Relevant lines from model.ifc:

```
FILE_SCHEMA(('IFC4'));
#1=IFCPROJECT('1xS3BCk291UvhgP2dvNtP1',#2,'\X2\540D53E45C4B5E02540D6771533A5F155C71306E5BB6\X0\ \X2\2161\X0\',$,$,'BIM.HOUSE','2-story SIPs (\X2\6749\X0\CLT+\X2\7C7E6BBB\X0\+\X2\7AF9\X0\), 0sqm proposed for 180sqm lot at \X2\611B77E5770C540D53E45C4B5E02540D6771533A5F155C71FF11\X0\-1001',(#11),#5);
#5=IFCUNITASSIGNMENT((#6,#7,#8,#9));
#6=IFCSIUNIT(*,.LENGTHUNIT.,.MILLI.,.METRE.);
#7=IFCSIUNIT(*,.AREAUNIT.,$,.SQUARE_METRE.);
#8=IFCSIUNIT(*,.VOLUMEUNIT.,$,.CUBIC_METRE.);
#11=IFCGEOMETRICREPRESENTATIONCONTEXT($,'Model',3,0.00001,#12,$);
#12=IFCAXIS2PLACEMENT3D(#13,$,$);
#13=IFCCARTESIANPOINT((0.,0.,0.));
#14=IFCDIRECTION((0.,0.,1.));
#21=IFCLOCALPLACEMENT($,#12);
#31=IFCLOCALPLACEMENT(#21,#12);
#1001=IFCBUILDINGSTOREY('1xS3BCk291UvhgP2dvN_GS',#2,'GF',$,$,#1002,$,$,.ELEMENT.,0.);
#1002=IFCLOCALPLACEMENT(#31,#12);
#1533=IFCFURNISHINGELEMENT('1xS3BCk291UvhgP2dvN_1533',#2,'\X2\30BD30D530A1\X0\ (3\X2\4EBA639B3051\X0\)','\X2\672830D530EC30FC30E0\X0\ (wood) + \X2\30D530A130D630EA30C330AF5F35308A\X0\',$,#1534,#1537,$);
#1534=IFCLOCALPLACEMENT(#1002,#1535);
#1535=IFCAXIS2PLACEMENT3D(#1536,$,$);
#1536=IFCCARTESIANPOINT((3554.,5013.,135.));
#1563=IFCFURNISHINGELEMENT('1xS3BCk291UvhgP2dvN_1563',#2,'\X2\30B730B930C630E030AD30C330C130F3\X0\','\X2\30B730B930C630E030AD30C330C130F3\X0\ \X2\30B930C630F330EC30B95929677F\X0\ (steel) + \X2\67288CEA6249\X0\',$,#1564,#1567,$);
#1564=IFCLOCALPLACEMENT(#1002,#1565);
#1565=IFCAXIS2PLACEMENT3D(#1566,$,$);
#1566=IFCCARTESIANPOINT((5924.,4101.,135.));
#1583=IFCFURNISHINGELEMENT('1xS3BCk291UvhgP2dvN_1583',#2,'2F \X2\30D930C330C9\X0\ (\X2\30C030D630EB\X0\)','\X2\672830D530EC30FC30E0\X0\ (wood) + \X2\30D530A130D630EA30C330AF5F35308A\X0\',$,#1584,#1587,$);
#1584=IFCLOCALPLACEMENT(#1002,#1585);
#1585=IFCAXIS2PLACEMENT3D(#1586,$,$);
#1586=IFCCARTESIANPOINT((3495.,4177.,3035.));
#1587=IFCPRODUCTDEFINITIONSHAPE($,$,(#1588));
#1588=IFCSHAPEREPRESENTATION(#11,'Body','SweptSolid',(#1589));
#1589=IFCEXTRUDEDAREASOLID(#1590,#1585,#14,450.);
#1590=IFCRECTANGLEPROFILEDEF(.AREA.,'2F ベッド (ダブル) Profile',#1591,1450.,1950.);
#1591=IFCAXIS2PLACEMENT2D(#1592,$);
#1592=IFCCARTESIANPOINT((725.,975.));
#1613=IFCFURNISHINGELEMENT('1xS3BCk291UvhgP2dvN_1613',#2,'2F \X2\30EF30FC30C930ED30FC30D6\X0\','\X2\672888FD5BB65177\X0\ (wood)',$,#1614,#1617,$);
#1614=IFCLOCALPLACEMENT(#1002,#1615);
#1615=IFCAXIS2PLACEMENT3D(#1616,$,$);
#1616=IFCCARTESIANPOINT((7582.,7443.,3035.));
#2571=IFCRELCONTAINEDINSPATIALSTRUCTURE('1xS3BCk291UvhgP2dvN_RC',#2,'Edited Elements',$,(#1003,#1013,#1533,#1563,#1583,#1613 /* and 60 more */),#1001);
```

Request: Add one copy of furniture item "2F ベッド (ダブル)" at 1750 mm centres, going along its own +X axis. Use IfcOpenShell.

```python
import ifcopenshell
import ifcopenshell.api.geometry
import ifcopenshell.api.root
import ifcopenshell.util.element
import ifcopenshell.util.placement
import ifcopenshell.util.unit

model = ifcopenshell.open("model.ifc")
unit_scale = ifcopenshell.util.unit.calculate_unit_scale(model)


def reuse_history(source, copy):
    """copy_class also copies each property set's owner history, people and application; keep the originals."""
    for rel in copy.IsDefinedBy:
        if rel.is_a("IfcRelDefinesByProperties") and (history := rel.RelatingPropertyDefinition.OwnerHistory):
            rel.RelatingPropertyDefinition.OwnerHistory = source.OwnerHistory
            ifcopenshell.util.element.remove_deep2(model, history)


source = model.by_guid("1xS3BCk291UvhgP2dvN_1583")
base = ifcopenshell.util.placement.get_local_placement(source.ObjectPlacement)
step = base[:3, 0] * 1.75 / unit_scale

for i in range(1, 2):
    copy = ifcopenshell.api.root.copy_class(model, product=source)
    copy.Representation = ifcopenshell.util.element.copy_deep(
        model, source.Representation, exclude=["IfcGeometricRepresentationContext", "IfcRepresentationMap"]
    )
    reuse_history(source, copy)
    matrix = base.copy()
    matrix[:3, 3] += i * step
    print("added at", matrix[:3, 3].round(3) + 0.0)
    ifcopenshell.api.geometry.edit_object_placement(model, product=copy, matrix=matrix, is_si=False)

model.write("model_rev.ifc")
```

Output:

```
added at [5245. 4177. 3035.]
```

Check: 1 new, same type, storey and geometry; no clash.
